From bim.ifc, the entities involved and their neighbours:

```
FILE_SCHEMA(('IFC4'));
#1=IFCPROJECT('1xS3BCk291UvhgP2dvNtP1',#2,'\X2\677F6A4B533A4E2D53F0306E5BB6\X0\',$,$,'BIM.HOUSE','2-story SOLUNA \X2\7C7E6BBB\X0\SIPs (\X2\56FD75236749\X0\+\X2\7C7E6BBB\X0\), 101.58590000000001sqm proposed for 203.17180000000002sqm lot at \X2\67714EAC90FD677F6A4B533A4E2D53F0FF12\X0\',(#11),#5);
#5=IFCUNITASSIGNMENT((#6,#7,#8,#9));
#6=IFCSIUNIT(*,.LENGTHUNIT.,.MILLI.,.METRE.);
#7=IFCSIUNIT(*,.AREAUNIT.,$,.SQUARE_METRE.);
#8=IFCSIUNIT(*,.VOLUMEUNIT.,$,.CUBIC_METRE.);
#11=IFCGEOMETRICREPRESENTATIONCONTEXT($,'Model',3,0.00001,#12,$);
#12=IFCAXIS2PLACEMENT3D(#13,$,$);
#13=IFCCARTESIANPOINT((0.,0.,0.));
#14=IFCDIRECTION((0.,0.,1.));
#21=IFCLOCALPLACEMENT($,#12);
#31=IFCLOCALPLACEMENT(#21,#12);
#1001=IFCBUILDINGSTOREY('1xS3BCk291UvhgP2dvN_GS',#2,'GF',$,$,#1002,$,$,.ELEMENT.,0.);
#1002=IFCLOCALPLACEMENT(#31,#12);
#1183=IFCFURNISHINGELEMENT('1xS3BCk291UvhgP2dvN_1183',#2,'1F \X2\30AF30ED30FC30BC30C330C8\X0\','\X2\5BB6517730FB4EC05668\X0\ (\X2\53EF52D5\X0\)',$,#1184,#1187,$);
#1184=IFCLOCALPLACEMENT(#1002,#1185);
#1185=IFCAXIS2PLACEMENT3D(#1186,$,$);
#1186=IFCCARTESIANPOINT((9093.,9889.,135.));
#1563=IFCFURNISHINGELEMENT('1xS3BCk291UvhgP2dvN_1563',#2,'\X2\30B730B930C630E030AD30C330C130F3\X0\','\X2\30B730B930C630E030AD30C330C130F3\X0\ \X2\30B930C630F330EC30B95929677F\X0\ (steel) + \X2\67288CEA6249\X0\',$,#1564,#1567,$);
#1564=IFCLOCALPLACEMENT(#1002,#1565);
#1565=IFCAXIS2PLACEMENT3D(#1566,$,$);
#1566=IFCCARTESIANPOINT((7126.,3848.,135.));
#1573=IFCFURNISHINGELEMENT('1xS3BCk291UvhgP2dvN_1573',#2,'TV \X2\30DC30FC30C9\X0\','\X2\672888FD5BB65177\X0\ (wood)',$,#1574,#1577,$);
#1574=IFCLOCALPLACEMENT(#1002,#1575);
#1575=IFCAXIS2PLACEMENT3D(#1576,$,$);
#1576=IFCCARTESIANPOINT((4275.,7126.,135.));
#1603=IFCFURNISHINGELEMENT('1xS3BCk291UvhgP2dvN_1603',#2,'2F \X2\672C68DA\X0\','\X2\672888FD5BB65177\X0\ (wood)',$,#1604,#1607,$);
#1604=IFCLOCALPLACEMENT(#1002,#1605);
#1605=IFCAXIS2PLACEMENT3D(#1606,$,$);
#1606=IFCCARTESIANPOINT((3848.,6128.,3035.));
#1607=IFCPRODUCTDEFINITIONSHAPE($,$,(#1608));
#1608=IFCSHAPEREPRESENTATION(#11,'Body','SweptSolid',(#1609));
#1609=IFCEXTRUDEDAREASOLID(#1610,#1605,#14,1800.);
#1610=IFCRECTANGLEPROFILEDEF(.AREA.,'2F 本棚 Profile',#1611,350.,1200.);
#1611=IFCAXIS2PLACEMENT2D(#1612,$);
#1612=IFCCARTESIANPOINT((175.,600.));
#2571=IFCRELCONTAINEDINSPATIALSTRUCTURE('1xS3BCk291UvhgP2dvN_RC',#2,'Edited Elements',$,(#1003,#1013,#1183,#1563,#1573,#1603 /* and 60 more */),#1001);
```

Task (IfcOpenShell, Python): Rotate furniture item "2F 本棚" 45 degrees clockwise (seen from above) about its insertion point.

```python
import ifcopenshell
import ifcopenshell.api.geometry
import ifcopenshell.util.placement

model = ifcopenshell.open("bim.ifc")

item = model.by_id(1603)
matrix = ifcopenshell.util.placement.get_local_placement(item.ObjectPlacement)
matrix = matrix @ ifcopenshell.util.placement.rotation(-45, "Z")
ifcopenshell.api.geometry.edit_object_placement(model, product=item, matrix=matrix, is_si=False)

print(ifcopenshell.util.placement.get_local_placement(item.ObjectPlacement).round(3) + 0.0)

model.write("bim_updated.ifc")
```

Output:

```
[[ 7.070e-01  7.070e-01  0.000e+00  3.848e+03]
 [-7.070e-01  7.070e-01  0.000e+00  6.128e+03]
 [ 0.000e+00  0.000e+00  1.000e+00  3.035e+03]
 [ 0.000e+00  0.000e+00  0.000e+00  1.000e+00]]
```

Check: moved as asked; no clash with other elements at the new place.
